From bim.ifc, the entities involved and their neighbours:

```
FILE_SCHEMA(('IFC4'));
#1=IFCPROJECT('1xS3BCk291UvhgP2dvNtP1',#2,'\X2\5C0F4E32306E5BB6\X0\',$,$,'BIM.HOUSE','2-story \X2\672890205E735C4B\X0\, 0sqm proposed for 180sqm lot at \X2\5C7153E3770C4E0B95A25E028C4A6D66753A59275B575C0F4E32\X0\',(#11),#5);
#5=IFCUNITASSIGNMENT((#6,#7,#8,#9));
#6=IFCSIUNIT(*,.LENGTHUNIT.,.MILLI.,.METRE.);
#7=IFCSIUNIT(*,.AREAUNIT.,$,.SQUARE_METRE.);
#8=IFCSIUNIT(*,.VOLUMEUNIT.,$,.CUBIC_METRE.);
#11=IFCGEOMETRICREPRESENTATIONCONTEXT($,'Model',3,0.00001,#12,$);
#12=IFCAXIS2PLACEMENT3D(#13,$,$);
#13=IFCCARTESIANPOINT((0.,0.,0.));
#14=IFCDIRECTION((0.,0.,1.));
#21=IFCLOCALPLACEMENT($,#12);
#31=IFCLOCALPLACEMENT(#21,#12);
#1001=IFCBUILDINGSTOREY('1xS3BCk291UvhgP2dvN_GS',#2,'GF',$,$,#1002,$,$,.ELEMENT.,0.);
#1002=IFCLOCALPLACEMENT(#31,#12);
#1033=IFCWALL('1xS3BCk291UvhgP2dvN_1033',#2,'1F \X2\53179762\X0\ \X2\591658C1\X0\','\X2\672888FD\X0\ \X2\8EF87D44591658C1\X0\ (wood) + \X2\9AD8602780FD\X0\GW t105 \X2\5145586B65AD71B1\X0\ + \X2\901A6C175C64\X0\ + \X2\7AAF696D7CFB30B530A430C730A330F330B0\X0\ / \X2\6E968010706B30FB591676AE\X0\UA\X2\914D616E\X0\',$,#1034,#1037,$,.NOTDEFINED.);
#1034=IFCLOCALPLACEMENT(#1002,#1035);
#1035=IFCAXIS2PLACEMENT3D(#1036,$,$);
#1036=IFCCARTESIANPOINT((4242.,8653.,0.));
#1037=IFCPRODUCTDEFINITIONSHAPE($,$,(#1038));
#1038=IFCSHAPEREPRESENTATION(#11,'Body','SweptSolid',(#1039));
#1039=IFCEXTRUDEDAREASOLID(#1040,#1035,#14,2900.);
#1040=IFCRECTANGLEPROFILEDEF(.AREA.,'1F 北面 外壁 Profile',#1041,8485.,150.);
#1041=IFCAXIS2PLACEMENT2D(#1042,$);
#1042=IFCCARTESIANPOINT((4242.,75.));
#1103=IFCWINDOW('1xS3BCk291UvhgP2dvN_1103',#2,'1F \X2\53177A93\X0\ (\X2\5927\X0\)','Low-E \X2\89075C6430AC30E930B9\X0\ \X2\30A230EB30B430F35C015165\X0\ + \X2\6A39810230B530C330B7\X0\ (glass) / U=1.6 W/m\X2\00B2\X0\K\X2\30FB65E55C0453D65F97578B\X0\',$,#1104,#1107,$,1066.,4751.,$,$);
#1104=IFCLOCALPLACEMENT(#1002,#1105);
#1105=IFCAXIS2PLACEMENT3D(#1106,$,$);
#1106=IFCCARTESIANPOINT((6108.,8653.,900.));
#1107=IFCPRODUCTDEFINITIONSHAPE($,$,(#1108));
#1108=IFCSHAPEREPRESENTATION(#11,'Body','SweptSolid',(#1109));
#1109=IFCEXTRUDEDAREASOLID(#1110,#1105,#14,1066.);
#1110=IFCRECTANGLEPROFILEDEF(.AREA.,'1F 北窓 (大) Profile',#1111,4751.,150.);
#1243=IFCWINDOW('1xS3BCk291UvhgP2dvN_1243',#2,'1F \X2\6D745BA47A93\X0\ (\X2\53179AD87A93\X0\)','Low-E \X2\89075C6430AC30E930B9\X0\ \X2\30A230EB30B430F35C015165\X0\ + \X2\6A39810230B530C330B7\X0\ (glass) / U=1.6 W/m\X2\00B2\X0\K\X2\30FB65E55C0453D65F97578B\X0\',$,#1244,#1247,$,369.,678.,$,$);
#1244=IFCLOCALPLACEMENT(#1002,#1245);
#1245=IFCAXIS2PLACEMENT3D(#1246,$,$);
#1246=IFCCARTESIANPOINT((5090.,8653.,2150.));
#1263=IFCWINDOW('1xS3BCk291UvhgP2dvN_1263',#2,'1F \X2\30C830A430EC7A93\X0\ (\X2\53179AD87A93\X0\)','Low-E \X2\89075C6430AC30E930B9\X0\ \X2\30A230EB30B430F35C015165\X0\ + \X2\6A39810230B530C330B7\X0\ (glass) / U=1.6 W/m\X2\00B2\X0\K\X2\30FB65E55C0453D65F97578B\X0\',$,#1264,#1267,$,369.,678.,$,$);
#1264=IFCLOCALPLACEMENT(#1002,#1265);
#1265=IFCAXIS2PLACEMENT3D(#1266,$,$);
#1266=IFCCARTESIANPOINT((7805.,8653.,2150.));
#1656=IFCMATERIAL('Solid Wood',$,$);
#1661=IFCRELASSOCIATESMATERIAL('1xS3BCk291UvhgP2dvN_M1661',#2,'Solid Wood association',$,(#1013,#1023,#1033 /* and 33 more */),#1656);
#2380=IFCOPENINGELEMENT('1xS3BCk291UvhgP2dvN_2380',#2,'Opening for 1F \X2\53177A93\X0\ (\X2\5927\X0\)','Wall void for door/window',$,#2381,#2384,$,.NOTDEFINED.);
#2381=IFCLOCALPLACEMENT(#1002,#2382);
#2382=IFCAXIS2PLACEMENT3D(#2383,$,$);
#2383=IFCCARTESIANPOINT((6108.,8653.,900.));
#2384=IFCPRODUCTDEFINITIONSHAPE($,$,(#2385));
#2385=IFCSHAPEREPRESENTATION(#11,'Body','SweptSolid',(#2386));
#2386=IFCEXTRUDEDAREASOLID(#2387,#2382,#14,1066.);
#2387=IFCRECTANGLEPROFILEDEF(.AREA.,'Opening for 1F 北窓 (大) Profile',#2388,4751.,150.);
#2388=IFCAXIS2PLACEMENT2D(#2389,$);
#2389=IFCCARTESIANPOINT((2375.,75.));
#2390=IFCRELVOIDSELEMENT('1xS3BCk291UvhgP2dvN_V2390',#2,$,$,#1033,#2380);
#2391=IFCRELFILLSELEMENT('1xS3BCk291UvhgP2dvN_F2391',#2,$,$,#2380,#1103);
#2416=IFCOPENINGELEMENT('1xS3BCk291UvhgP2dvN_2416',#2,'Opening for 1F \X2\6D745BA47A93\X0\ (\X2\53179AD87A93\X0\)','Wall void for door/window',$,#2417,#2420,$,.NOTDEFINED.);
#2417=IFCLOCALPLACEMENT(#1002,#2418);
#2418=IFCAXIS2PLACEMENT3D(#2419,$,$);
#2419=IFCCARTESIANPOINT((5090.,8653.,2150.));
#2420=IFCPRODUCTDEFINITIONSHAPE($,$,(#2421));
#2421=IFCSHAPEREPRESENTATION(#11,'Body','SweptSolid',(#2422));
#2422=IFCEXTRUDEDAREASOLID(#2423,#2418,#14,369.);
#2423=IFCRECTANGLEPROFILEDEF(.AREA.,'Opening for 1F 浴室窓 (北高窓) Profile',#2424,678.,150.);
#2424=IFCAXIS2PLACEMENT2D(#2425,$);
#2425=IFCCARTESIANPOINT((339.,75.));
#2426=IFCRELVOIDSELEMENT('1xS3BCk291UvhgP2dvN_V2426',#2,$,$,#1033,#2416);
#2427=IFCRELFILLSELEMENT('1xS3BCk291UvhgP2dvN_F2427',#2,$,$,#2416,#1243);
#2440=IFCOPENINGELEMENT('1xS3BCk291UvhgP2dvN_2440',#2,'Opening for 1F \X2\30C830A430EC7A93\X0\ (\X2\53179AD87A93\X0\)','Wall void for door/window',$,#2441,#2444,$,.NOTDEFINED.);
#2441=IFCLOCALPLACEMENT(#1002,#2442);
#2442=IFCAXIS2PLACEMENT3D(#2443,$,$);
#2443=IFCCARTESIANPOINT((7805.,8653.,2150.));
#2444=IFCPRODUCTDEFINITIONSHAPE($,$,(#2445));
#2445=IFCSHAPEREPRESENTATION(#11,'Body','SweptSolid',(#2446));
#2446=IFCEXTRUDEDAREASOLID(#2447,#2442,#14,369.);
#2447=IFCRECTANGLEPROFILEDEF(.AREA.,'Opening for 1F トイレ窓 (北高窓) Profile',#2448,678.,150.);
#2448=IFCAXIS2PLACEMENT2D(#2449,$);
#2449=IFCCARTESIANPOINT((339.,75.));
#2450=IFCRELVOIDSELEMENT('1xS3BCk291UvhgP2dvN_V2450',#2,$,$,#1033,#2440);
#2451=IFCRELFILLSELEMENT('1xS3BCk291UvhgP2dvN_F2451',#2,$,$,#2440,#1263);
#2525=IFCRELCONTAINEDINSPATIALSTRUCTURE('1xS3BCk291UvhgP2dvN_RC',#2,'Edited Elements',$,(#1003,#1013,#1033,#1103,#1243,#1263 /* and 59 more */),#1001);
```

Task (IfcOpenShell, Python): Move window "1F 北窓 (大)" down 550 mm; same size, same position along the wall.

```python
import numpy as np
import ifcopenshell
import ifcopenshell.api.geometry
import ifcopenshell.util.placement
import ifcopenshell.util.unit

model = ifcopenshell.open("bim.ifc")
unit_scale = ifcopenshell.util.unit.calculate_unit_scale(model)

window = model.by_guid("1xS3BCk291UvhgP2dvN_1103")
opening = window.FillsVoids[0].RelatingOpeningElement
dz = -0.55 / unit_scale

shift = np.array([0.0, 0.0, dz])
# The window is not placed relative to its opening, so move both.
for product in (opening, window):
    matrix = ifcopenshell.util.placement.get_local_placement(product.ObjectPlacement)
    matrix[:3, 3] += shift
    ifcopenshell.api.geometry.edit_object_placement(model, product=product, matrix=matrix, is_si=False)

print(f"moved by {dz * unit_scale:+.3f} m")

model.write("bim_updated.ifc")
```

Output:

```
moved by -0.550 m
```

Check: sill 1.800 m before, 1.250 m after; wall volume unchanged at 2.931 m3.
